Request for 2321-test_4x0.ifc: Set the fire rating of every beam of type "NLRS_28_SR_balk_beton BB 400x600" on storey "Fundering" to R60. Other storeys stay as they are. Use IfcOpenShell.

First a look at what the model holds.

```python
import ifcopenshell
import ifcopenshell.util.element

model = ifcopenshell.open("2321-test_4x0.ifc")
print(model.schema)
storey = next(s for s in model.by_type("IfcBuildingStorey") if s.Name == "Fundering")
beams = [e for e in ifcopenshell.util.element.get_decomposition(storey) if e.is_a("IfcBeam")]
seen = {}
for e in beams:
    element_type = ifcopenshell.util.element.get_type(e)
    key = (element_type.Name if element_type != e and element_type else None, ifcopenshell.util.element.get_pset(e, "Pset_BeamCommon", "FireRating"))
    seen[key] = seen.get(key, 0) + 1
for (name, value), count in sorted(seen.items(), key=str):
    print(count, "x", name, "|", value)
```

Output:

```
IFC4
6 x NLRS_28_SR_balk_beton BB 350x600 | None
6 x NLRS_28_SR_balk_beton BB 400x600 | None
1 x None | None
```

```python
import ifcopenshell
import ifcopenshell.api.pset
import ifcopenshell.util.element

model = ifcopenshell.open("2321-test_4x0.ifc")

storey = next(s for s in model.by_type("IfcBuildingStorey") if s.Name == "Fundering")
beams = [e for e in ifcopenshell.util.element.get_decomposition(storey) if e.is_a("IfcBeam")]

count = 0
for e in beams:
    element_type = ifcopenshell.util.element.get_type(e)
    if element_type in (None, e) or element_type.Name != "NLRS_28_SR_balk_beton BB 400x600":
        continue
    # add_pset returns the element's existing set when there is one.
    pset = ifcopenshell.api.pset.add_pset(model, product=e, name="Pset_BeamCommon")
    ifcopenshell.api.pset.edit_pset(model, pset=pset, properties={"FireRating": "R60"})
    count += 1

print(count, "beams updated")

model.write("2321-test_4x0-out.ifc")
```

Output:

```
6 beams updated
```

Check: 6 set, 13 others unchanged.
